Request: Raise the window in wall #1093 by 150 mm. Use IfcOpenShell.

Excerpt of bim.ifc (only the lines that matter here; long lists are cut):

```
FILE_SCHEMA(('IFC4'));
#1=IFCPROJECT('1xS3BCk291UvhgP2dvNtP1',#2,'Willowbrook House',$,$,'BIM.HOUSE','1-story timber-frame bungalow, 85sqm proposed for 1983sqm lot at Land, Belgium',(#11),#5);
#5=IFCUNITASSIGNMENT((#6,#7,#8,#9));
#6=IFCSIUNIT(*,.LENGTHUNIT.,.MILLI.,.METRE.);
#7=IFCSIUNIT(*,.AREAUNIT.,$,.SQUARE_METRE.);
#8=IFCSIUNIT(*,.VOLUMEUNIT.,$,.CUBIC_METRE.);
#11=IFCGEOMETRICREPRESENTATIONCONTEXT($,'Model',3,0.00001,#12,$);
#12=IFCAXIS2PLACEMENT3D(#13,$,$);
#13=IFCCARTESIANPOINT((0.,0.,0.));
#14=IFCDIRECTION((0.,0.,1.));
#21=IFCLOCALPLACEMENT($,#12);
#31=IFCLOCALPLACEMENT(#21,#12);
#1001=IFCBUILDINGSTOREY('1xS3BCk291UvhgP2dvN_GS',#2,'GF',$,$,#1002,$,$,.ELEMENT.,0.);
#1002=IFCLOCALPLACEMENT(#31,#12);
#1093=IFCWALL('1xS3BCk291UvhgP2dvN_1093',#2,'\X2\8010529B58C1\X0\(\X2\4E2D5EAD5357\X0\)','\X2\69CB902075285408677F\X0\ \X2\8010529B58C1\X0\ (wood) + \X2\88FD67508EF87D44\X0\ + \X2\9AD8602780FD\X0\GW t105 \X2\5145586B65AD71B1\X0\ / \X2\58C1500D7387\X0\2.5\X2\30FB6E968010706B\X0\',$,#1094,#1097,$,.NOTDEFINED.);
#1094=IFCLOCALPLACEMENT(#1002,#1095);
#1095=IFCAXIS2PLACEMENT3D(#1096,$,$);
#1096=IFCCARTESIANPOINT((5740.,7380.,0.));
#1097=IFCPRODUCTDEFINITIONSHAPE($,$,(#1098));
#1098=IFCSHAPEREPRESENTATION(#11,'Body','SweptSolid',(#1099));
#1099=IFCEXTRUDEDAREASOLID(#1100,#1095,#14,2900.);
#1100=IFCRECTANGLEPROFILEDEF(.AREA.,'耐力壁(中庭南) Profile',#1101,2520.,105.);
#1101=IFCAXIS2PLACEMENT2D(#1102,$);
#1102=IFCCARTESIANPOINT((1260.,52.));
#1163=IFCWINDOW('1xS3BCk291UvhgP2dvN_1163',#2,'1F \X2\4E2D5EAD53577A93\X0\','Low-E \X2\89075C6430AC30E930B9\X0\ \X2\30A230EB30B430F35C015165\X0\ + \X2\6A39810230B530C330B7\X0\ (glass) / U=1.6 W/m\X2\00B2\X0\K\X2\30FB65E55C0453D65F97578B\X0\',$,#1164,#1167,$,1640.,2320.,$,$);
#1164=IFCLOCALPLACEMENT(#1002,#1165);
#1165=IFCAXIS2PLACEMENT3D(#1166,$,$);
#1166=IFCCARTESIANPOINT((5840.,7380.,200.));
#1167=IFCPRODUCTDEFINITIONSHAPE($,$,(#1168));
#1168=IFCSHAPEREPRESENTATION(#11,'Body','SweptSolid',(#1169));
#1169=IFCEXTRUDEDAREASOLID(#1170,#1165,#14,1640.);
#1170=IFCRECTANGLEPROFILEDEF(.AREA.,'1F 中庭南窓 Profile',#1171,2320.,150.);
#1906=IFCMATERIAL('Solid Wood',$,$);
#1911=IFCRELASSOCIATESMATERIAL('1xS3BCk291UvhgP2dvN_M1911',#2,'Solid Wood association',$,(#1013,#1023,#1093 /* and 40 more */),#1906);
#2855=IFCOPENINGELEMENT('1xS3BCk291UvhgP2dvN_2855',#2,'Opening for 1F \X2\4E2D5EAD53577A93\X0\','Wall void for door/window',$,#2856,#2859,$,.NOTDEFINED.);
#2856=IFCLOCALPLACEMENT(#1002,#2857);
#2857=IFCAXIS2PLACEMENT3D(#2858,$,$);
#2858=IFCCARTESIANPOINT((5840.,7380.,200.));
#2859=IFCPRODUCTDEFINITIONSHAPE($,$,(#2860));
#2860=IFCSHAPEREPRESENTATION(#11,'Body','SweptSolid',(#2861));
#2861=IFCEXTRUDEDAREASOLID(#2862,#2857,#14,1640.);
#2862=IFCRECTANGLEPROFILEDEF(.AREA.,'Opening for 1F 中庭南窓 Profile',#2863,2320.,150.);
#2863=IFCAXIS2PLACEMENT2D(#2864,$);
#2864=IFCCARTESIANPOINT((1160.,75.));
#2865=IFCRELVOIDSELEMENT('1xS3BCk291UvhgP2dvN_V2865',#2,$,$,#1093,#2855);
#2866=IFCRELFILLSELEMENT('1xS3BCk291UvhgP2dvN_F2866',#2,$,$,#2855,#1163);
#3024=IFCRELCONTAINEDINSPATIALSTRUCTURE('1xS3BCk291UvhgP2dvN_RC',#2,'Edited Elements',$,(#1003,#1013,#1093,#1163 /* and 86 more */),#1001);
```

```python
import numpy as np
import ifcopenshell
import ifcopenshell.api.geometry
import ifcopenshell.util.placement
import ifcopenshell.util.unit

model = ifcopenshell.open("bim.ifc")
unit_scale = ifcopenshell.util.unit.calculate_unit_scale(model)

window = model.by_guid("1xS3BCk291UvhgP2dvN_1163")
opening = window.FillsVoids[0].RelatingOpeningElement
dz = 0.15 / unit_scale

shift = np.array([0.0, 0.0, dz])
# The window is not placed relative to its opening, so move both.
for product in (opening, window):
    matrix = ifcopenshell.util.placement.get_local_placement(product.ObjectPlacement)
    matrix[:3, 3] += shift
    ifcopenshell.api.geometry.edit_object_placement(model, product=product, matrix=matrix, is_si=False)

print(f"moved by {dz * unit_scale:+.3f} m")

model.write("bim_rev.ifc")
```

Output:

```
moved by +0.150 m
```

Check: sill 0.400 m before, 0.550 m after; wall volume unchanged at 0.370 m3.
